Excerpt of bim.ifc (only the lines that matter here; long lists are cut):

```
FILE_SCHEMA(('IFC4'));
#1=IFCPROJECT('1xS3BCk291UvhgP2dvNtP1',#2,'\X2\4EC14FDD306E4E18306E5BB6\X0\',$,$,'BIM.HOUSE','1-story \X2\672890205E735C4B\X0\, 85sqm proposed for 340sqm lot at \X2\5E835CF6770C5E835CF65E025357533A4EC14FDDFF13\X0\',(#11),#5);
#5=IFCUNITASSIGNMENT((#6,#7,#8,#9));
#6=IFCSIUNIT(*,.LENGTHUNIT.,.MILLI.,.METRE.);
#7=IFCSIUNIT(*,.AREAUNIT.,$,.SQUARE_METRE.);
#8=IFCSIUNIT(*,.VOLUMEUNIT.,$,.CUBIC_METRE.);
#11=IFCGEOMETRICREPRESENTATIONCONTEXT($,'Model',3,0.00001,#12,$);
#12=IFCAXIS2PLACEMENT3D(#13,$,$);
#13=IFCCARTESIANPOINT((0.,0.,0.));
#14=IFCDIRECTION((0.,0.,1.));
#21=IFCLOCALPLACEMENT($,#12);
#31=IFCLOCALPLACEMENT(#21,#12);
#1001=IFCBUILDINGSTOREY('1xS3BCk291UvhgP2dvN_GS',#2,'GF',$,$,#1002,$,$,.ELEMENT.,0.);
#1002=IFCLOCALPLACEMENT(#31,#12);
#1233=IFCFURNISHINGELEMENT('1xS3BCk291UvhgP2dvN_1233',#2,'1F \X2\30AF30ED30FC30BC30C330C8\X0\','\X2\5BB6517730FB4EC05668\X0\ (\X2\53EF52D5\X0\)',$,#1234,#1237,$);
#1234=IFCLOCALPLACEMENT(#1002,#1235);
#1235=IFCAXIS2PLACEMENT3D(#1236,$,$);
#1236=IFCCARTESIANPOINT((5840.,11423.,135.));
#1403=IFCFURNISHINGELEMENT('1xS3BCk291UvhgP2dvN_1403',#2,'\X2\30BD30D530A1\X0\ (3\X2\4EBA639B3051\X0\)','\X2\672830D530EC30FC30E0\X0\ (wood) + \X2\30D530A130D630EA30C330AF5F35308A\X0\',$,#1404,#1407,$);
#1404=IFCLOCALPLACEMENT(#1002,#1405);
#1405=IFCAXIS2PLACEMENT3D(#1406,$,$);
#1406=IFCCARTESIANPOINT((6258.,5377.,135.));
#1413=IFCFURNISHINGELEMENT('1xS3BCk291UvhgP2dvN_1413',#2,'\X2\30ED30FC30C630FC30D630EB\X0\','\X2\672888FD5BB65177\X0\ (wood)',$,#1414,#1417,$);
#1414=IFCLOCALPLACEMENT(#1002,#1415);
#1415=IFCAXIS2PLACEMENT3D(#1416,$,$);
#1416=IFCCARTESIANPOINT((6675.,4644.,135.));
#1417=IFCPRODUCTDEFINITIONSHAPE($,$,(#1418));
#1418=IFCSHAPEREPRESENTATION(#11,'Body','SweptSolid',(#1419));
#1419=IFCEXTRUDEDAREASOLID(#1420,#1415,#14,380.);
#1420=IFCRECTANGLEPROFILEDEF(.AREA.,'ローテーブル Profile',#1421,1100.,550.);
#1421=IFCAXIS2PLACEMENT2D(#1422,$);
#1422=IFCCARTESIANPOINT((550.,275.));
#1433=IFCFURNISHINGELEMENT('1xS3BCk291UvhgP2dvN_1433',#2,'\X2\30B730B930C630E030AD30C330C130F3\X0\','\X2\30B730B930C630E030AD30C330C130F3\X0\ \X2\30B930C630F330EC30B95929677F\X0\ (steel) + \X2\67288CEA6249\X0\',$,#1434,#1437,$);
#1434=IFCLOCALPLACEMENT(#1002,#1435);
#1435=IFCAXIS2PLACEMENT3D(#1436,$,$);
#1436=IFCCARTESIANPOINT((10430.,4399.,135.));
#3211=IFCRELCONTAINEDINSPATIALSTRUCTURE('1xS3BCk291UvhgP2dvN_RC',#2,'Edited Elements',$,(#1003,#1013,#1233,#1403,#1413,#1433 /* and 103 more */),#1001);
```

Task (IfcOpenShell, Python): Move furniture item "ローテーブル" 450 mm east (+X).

```python
import ifcopenshell
import ifcopenshell.api.geometry
import ifcopenshell.util.placement

model = ifcopenshell.open("bim.ifc")

item = model.by_guid("1xS3BCk291UvhgP2dvN_1413")
matrix = ifcopenshell.util.placement.get_local_placement(item.ObjectPlacement)
matrix[0, 3] += 450.0
ifcopenshell.api.geometry.edit_object_placement(model, product=item, matrix=matrix, is_si=False)

print(ifcopenshell.util.placement.get_local_placement(item.ObjectPlacement).round(3) + 0.0)

model.write("bim-out.ifc")
```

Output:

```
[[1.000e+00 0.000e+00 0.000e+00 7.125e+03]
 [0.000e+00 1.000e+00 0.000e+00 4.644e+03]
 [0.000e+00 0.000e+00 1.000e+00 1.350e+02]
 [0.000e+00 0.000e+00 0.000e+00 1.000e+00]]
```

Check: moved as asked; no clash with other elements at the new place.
